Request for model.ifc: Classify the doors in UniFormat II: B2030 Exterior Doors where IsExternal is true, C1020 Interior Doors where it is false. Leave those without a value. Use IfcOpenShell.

First a look at what the model holds.

```python
import ifcopenshell
import ifcopenshell.util.element

model = ifcopenshell.open("model.ifc")
print(model.schema)
print("classifications:", [c.Name for c in model.by_type("IfcClassification")])
values = [ifcopenshell.util.element.get_pset(e, "Pset_DoorCommon", "IsExternal") for e in model.by_type("IfcDoor")]
for value in (True, False, None):
    print("IsExternal", value, values.count(value))
```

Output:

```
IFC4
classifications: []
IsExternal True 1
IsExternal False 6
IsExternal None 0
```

```python
import ifcopenshell
import ifcopenshell.api.classification
import ifcopenshell.util.element

model = ifcopenshell.open("model.ifc")

system = ifcopenshell.api.classification.add_classification(model, classification="UniFormat II")

doors = model.by_type("IfcDoor")
external = {e: ifcopenshell.util.element.get_pset(e, "Pset_DoorCommon", "IsExternal") for e in doors}
for flag, code, name in ((True, "B2030", "Exterior Doors"), (False, "C1020", "Interior Doors")):
    products = [e for e in doors if external[e] is flag]
    ifcopenshell.api.classification.add_reference(
        model, products=products, classification=system, identification=code, name=name
    )
    print(code, len(products))

model.write("model_rev.ifc")
```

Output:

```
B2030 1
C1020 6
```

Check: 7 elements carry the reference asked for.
